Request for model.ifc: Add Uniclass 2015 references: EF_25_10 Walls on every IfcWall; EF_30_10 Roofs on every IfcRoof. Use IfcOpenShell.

First a look at what the model holds.

```python
import ifcopenshell

model = ifcopenshell.open("model.ifc")
print(model.schema)
print("classifications:", [c.Name for c in model.by_type("IfcClassification")])
for ifc_class in ("IfcDoor", "IfcRoof", "IfcStair", "IfcWall", "IfcWindow"):
    print(ifc_class, len(model.by_type(ifc_class)))
```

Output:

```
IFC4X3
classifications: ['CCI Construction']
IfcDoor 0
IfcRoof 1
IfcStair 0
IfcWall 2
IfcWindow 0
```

```python
import ifcopenshell
import ifcopenshell.api.classification

model = ifcopenshell.open("model.ifc")

system = ifcopenshell.api.classification.add_classification(model, classification="Uniclass 2015")

codes = {
    "IfcWall": ("EF_25_10", "Walls"),
    "IfcRoof": ("EF_30_10", "Roofs"),
}
for ifc_class, (code, name) in codes.items():
    products = model.by_type(ifc_class)
    ifcopenshell.api.classification.add_reference(
        model, products=products, classification=system, identification=code, name=name
    )
    print(code, len(products))

model.write("model_rev.ifc")
```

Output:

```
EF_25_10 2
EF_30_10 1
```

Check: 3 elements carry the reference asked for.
